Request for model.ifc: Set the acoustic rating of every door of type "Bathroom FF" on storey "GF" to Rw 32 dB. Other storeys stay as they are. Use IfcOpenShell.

First a look at what the model holds.

```python
import ifcopenshell
import ifcopenshell.util.element

model = ifcopenshell.open("model.ifc")
print(model.schema)
storey = next(s for s in model.by_type("IfcBuildingStorey") if s.Name == "GF")
doors = [e for e in ifcopenshell.util.element.get_decomposition(storey) if e.is_a("IfcDoor")]
seen = {}
for e in doors:
    element_type = ifcopenshell.util.element.get_type(e)
    key = (element_type.Name if element_type != e and element_type else None, ifcopenshell.util.element.get_pset(e, "Pset_DoorCommon", "AcousticRating"))
    seen[key] = seen.get(key, 0) + 1
for (name, value), count in sorted(seen.items(), key=str):
    print(count, "x", name, "|", value)
```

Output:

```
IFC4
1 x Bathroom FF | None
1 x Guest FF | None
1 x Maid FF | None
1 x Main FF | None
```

```python
import ifcopenshell
import ifcopenshell.api.pset
import ifcopenshell.util.element

model = ifcopenshell.open("model.ifc")

storey = next(s for s in model.by_type("IfcBuildingStorey") if s.Name == "GF")
doors = [e for e in ifcopenshell.util.element.get_decomposition(storey) if e.is_a("IfcDoor")]

count = 0
for e in doors:
    element_type = ifcopenshell.util.element.get_type(e)
    if element_type in (None, e) or element_type.Name != "Bathroom FF":
        continue
    # add_pset returns the element's existing set when there is one.
    pset = ifcopenshell.api.pset.add_pset(model, product=e, name="Pset_DoorCommon")
    ifcopenshell.api.pset.edit_pset(model, pset=pset, properties={"AcousticRating": "Rw 32 dB"})
    count += 1

print(count, "doors updated")

model.write("model-out.ifc")
```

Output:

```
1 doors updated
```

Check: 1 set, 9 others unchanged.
